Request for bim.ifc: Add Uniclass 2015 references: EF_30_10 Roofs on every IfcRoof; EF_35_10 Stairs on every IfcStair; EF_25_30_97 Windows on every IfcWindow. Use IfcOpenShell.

First a look at what the model holds.

```python
import ifcopenshell

model = ifcopenshell.open("bim.ifc")
print(model.schema)
print("classifications:", [c.Name for c in model.by_type("IfcClassification")])
for ifc_class in ("IfcDoor", "IfcRoof", "IfcStair", "IfcWall", "IfcWindow"):
    print(ifc_class, len(model.by_type(ifc_class)))
```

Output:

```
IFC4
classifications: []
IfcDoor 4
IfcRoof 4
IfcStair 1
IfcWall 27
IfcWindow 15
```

```python
import ifcopenshell
import ifcopenshell.api.classification

model = ifcopenshell.open("bim.ifc")

system = ifcopenshell.api.classification.add_classification(model, classification="Uniclass 2015")

codes = {
    "IfcRoof": ("EF_30_10", "Roofs"),
    "IfcStair": ("EF_35_10", "Stairs"),
    "IfcWindow": ("EF_25_30_97", "Windows"),
}
for ifc_class, (code, name) in codes.items():
    products = model.by_type(ifc_class)
    ifcopenshell.api.classification.add_reference(
        model, products=products, classification=system, identification=code, name=name
    )
    print(code, len(products))

model.write("bim_v2.ifc")
```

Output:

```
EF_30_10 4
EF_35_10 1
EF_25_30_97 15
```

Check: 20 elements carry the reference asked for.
